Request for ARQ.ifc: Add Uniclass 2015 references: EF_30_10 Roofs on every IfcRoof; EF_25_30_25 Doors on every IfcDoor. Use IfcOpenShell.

First a look at what the model holds.

```python
import ifcopenshell

model = ifcopenshell.open("ARQ.ifc")
print(model.schema)
print("classifications:", [c.Name for c in model.by_type("IfcClassification")])
for ifc_class in ("IfcDoor", "IfcRoof", "IfcStair", "IfcWall", "IfcWindow"):
    print(ifc_class, len(model.by_type(ifc_class)))
```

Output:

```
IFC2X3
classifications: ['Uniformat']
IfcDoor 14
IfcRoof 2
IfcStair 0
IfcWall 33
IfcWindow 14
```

```python
import ifcopenshell
import ifcopenshell.api.classification

model = ifcopenshell.open("ARQ.ifc")

# IFC2X3 requires Source and Edition and has no link from the project to the system.
system = model.create_entity("IfcClassification", Source="NBS", Edition="2015", Name="Uniclass 2015")

codes = {
    "IfcRoof": ("EF_30_10", "Roofs"),
    "IfcDoor": ("EF_25_30_25", "Doors"),
}
for ifc_class, (code, name) in codes.items():
    products = model.by_type(ifc_class)
    ifcopenshell.api.classification.add_reference(
        model, products=products, classification=system, identification=code, name=name
    )
    print(code, len(products))

model.write("ARQ_rev.ifc")
```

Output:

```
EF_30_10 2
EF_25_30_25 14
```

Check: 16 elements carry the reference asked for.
